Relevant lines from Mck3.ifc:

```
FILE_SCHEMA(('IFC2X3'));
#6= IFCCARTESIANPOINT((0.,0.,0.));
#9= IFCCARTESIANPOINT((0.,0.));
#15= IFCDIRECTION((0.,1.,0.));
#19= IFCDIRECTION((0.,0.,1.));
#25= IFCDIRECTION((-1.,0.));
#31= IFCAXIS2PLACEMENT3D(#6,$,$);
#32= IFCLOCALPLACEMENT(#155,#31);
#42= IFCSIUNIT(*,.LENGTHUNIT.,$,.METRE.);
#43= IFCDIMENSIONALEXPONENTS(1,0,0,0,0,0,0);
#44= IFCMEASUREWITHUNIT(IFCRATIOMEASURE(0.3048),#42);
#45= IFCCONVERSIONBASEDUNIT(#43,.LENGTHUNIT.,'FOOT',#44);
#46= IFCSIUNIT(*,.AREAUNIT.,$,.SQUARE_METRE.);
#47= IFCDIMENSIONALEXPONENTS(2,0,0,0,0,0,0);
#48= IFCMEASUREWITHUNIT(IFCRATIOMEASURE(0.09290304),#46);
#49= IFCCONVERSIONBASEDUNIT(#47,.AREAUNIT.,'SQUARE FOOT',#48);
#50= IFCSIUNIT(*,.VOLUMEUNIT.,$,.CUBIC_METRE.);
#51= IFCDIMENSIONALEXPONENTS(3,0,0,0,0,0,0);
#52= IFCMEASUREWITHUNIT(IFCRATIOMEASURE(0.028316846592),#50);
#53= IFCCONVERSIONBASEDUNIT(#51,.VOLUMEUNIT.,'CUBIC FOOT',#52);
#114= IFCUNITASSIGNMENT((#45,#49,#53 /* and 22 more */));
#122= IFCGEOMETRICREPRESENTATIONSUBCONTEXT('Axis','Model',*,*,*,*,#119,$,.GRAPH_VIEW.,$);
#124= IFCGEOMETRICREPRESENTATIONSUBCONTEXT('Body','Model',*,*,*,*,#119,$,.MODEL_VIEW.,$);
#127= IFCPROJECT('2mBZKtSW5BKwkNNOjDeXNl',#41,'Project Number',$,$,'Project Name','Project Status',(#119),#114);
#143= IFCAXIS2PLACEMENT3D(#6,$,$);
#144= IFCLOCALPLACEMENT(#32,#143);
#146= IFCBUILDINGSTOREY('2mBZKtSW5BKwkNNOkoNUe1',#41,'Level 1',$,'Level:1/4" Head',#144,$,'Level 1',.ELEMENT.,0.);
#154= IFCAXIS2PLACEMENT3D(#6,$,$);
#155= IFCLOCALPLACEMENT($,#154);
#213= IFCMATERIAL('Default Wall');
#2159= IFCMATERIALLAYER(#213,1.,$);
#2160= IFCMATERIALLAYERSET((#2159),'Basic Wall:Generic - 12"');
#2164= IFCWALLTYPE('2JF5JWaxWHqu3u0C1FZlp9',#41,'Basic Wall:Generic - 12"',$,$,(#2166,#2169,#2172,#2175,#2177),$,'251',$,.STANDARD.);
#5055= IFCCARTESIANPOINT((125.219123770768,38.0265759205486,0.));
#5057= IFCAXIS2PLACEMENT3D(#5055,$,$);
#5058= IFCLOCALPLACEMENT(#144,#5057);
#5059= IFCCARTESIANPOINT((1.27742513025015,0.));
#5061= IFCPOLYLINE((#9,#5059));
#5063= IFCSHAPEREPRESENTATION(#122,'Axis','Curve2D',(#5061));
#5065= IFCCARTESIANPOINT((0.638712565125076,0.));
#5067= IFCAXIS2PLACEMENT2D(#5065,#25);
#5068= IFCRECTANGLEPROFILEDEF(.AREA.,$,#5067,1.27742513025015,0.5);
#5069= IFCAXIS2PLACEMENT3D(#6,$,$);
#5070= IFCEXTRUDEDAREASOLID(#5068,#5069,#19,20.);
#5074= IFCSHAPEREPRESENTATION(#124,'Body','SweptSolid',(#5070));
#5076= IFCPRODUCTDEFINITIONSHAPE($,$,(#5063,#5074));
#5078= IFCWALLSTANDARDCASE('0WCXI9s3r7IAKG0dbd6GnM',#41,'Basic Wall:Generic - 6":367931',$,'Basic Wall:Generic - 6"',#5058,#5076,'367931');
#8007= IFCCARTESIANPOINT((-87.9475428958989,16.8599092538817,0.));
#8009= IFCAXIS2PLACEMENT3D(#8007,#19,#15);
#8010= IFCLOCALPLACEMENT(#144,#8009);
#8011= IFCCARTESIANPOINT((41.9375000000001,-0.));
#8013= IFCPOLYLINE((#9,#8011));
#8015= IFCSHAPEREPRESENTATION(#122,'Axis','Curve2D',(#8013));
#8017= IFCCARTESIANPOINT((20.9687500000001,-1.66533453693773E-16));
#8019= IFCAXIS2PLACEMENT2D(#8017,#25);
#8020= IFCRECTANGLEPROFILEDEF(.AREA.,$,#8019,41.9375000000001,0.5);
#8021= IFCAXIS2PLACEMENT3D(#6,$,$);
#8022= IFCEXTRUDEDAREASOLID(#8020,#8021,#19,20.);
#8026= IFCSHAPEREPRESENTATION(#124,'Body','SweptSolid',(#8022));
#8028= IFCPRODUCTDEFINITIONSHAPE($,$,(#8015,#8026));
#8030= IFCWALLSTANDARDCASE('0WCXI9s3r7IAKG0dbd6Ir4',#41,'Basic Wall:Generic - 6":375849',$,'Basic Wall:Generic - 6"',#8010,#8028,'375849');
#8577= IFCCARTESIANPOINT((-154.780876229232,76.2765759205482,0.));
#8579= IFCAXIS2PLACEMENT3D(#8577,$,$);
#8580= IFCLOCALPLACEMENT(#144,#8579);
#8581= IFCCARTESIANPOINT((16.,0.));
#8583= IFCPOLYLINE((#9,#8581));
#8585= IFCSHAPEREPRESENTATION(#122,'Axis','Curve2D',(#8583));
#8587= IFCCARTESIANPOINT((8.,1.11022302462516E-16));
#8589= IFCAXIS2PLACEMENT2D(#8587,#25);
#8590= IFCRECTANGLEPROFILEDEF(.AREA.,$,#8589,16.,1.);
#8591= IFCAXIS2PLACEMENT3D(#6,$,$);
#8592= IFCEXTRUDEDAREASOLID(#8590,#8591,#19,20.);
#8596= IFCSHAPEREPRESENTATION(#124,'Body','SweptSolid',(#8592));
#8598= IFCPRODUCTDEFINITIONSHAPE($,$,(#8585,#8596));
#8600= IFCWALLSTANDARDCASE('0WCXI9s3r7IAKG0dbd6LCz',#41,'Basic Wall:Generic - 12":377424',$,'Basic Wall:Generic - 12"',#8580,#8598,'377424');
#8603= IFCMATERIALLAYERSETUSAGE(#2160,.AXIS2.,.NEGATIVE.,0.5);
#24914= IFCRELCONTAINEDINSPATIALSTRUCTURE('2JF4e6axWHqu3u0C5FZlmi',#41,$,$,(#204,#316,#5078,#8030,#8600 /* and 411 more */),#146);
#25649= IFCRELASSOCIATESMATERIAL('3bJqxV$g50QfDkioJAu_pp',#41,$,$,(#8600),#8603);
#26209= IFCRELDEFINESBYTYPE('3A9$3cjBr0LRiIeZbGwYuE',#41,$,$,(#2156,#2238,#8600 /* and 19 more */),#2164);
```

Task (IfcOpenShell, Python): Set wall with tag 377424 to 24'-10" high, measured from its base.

```python
import ifcopenshell
import ifcopenshell.geom
import ifcopenshell.util.representation
import ifcopenshell.util.shape
import ifcopenshell.util.unit

model = ifcopenshell.open("Mck3.ifc")
unit_scale = ifcopenshell.util.unit.calculate_unit_scale(model)
settings = ifcopenshell.geom.settings()


def volume(element):
    """Net volume in cubic metres, openings subtracted."""
    shape = ifcopenshell.geom.create_shape(settings, element)
    return ifcopenshell.util.shape.get_volume(shape.geometry)


wall = model.by_id(8600)
before = volume(wall)

body = ifcopenshell.util.representation.get_representation(wall, "Model", "Body")
solid = body.Items[0]
old_height = solid.Depth
solid.Depth = 298 * 0.0254 / unit_scale
after = volume(wall)

print(f"height {old_height:g} -> {solid.Depth:g}, volume {before:.3f} -> {after:.3f} m3")

model.write("Mck3_updated.ifc")
```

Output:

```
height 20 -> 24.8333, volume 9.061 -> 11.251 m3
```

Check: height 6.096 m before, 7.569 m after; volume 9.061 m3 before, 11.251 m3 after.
